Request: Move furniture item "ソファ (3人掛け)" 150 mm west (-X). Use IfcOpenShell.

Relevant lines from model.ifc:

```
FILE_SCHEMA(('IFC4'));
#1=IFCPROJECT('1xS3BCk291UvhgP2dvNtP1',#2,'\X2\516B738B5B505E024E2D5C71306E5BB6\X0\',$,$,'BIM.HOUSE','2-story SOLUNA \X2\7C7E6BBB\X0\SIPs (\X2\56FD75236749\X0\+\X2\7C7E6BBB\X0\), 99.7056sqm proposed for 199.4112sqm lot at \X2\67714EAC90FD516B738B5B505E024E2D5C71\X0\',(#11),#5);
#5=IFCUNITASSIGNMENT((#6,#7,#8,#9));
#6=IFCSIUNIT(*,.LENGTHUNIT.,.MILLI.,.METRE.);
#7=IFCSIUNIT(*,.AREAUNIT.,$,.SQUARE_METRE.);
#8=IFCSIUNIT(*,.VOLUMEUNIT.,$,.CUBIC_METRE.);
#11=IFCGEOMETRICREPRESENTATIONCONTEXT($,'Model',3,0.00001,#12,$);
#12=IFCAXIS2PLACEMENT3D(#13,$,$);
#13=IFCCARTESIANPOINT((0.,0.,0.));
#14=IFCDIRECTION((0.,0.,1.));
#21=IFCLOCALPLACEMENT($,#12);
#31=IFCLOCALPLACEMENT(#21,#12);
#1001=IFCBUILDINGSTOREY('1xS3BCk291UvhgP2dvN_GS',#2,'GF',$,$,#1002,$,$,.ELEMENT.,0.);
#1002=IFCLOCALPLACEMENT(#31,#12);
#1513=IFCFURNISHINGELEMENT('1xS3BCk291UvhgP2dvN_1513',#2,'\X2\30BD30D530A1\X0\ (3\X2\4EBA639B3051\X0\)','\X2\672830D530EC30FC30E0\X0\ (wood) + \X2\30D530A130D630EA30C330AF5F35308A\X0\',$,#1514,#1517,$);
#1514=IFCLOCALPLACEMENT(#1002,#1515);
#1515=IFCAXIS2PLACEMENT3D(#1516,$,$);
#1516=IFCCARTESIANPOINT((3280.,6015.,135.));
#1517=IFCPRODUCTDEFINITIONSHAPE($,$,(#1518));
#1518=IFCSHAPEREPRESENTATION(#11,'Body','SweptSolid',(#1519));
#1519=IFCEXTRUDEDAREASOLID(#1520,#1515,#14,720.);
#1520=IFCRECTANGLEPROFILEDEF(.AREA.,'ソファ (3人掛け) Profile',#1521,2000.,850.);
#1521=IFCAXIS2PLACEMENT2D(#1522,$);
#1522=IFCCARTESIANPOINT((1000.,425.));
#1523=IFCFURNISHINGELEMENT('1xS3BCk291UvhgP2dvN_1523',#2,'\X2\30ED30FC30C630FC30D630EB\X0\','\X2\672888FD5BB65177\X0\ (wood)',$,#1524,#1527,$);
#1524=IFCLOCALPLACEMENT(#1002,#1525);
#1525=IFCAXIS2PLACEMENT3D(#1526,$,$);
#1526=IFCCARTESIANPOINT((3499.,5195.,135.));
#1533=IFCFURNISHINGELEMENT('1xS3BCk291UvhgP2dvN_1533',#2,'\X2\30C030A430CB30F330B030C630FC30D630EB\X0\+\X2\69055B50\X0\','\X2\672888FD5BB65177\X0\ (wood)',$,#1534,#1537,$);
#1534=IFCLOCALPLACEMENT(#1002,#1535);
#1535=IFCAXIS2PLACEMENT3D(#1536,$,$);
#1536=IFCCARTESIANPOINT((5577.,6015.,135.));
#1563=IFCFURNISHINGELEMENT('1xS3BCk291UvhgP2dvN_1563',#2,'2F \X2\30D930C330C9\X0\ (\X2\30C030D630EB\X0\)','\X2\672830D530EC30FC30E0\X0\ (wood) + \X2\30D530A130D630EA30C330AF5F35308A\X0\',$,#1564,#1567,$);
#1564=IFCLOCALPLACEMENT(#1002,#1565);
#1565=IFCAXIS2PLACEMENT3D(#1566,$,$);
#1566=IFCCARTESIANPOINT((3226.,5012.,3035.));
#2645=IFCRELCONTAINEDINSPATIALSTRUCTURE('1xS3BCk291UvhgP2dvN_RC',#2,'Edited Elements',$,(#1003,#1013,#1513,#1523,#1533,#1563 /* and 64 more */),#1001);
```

```python
import ifcopenshell
import ifcopenshell.api.geometry
import ifcopenshell.util.placement

model = ifcopenshell.open("model.ifc")

item = model.by_id(1513)
matrix = ifcopenshell.util.placement.get_local_placement(item.ObjectPlacement)
matrix[0, 3] -= 150.0
ifcopenshell.api.geometry.edit_object_placement(model, product=item, matrix=matrix, is_si=False)

print(ifcopenshell.util.placement.get_local_placement(item.ObjectPlacement).round(3) + 0.0)

model.write("model-out.ifc")
```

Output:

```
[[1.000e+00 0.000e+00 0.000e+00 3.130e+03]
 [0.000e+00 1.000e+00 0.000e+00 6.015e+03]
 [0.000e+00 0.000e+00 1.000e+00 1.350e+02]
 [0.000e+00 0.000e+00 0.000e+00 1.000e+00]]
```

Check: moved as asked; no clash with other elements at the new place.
